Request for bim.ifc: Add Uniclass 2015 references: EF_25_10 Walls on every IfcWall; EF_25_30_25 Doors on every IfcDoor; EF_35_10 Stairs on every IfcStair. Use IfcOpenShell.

First a look at what the model holds.

```python
import ifcopenshell

model = ifcopenshell.open("bim.ifc")
print(model.schema)
print("classifications:", [c.Name for c in model.by_type("IfcClassification")])
for ifc_class in ("IfcDoor", "IfcRoof", "IfcStair", "IfcWall", "IfcWindow"):
    print(ifc_class, len(model.by_type(ifc_class)))
```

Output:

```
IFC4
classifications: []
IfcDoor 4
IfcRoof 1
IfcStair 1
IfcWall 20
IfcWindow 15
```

```python
import ifcopenshell
import ifcopenshell.api.classification

model = ifcopenshell.open("bim.ifc")

system = ifcopenshell.api.classification.add_classification(model, classification="Uniclass 2015")

codes = {
    "IfcWall": ("EF_25_10", "Walls"),
    "IfcDoor": ("EF_25_30_25", "Doors"),
    "IfcStair": ("EF_35_10", "Stairs"),
}
for ifc_class, (code, name) in codes.items():
    products = model.by_type(ifc_class)
    ifcopenshell.api.classification.add_reference(
        model, products=products, classification=system, identification=code, name=name
    )
    print(code, len(products))

model.write("bim_updated.ifc")
```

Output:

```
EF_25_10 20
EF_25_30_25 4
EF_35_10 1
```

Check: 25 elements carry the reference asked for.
